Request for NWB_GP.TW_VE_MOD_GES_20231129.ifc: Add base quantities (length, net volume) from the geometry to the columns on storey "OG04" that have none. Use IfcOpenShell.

First a look at what the model holds.

```python
import ifcopenshell
import ifcopenshell.util.element
import ifcopenshell.util.unit

model = ifcopenshell.open("NWB_GP.TW_VE_MOD_GES_20231129.ifc")
print(model.schema)
for unit_type in ("LENGTHUNIT", "AREAUNIT", "VOLUMEUNIT"):
    print(unit_type, ifcopenshell.util.unit.calculate_unit_scale(model, unit_type))
storey = next(s for s in model.by_type("IfcBuildingStorey") if s.Name == "OG04")
columns = [e for e in ifcopenshell.util.element.get_decomposition(storey) if e.is_a("IfcColumn")]
for e in sorted(columns, key=lambda e: e.id()):
    print(e.id(), e.is_a(), e.Name, list(ifcopenshell.util.element.get_psets(e, qtos_only=True)), sep=" | ")
```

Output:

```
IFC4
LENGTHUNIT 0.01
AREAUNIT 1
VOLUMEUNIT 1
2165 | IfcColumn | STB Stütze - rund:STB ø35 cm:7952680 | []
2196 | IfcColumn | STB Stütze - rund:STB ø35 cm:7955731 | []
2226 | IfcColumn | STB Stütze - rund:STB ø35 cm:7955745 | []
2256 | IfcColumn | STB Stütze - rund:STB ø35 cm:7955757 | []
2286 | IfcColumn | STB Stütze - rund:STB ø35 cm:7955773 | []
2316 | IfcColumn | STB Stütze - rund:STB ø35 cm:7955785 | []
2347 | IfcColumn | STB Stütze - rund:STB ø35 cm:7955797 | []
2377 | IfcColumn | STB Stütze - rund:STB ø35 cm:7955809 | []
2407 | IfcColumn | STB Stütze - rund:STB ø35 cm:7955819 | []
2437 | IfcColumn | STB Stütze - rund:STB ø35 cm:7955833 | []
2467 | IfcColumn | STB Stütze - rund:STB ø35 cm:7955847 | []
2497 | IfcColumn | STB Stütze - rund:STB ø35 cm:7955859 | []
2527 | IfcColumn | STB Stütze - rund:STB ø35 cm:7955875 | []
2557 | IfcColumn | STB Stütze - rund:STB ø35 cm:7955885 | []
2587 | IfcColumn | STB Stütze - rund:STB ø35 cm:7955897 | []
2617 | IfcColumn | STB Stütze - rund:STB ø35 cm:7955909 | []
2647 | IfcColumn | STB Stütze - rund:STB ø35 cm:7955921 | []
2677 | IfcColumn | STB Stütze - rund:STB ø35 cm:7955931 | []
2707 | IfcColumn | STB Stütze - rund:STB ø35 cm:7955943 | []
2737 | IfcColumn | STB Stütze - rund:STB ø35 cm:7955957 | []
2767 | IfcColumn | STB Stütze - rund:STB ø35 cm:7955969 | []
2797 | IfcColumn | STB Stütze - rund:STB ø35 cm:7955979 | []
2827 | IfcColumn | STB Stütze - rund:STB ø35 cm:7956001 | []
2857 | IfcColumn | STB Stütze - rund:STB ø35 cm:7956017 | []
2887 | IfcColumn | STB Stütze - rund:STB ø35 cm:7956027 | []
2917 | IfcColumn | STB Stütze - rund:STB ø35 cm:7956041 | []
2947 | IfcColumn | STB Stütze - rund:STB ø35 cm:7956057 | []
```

```python
import ifcopenshell
import ifcopenshell.api.pset
import ifcopenshell.geom
import ifcopenshell.util.element
import ifcopenshell.util.shape
import ifcopenshell.util.unit

model = ifcopenshell.open("NWB_GP.TW_VE_MOD_GES_20231129.ifc")
unit_scale = ifcopenshell.util.unit.calculate_unit_scale(model)
volume_scale = ifcopenshell.util.unit.calculate_unit_scale(model, "VOLUMEUNIT")
settings = ifcopenshell.geom.settings()

storey = next(s for s in model.by_type("IfcBuildingStorey") if s.Name == "OG04")
columns = [e for e in ifcopenshell.util.element.get_decomposition(storey) if e.is_a("IfcColumn")]

for e in sorted(columns, key=lambda e: e.id()):
    if ifcopenshell.util.element.get_psets(e, qtos_only=True, should_inherit=False):
        continue
    # Geometry comes back in metres, in the element's own axes.
    shape = ifcopenshell.geom.create_shape(settings, e)
    values = {
        "Length": ifcopenshell.util.shape.get_z(shape.geometry) / unit_scale,
        "NetVolume": ifcopenshell.util.shape.get_volume(shape.geometry) / volume_scale,
    }
    qto = ifcopenshell.api.pset.add_qto(model, product=e, name="Qto_ColumnBaseQuantities")
    ifcopenshell.api.pset.edit_qto(model, qto=qto, properties=values)
    print(e.id(), {k: round(v, 3) for k, v in values.items()})

model.write("NWB_GP.TW_VE_MOD_GES_20231129_v2.ifc")
```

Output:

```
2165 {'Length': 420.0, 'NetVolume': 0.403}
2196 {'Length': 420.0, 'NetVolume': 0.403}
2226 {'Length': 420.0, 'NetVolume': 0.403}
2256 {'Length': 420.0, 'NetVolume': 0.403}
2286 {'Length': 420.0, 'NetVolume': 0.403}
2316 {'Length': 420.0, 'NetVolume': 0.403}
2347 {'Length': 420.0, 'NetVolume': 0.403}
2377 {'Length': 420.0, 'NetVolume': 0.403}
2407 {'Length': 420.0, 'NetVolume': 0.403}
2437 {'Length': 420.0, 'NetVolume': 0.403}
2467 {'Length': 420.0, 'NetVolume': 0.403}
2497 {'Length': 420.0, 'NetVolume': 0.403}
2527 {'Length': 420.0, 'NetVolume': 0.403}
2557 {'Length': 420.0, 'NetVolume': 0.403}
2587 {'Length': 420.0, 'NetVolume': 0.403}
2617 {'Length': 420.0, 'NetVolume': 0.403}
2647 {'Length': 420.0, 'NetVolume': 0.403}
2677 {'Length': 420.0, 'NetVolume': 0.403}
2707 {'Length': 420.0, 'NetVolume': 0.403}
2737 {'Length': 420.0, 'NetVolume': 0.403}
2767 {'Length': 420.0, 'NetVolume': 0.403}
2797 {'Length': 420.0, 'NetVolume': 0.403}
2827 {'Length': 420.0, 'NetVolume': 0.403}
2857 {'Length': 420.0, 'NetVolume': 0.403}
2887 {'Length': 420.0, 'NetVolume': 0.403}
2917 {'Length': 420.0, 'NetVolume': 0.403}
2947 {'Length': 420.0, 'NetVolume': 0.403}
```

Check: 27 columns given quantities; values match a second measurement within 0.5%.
